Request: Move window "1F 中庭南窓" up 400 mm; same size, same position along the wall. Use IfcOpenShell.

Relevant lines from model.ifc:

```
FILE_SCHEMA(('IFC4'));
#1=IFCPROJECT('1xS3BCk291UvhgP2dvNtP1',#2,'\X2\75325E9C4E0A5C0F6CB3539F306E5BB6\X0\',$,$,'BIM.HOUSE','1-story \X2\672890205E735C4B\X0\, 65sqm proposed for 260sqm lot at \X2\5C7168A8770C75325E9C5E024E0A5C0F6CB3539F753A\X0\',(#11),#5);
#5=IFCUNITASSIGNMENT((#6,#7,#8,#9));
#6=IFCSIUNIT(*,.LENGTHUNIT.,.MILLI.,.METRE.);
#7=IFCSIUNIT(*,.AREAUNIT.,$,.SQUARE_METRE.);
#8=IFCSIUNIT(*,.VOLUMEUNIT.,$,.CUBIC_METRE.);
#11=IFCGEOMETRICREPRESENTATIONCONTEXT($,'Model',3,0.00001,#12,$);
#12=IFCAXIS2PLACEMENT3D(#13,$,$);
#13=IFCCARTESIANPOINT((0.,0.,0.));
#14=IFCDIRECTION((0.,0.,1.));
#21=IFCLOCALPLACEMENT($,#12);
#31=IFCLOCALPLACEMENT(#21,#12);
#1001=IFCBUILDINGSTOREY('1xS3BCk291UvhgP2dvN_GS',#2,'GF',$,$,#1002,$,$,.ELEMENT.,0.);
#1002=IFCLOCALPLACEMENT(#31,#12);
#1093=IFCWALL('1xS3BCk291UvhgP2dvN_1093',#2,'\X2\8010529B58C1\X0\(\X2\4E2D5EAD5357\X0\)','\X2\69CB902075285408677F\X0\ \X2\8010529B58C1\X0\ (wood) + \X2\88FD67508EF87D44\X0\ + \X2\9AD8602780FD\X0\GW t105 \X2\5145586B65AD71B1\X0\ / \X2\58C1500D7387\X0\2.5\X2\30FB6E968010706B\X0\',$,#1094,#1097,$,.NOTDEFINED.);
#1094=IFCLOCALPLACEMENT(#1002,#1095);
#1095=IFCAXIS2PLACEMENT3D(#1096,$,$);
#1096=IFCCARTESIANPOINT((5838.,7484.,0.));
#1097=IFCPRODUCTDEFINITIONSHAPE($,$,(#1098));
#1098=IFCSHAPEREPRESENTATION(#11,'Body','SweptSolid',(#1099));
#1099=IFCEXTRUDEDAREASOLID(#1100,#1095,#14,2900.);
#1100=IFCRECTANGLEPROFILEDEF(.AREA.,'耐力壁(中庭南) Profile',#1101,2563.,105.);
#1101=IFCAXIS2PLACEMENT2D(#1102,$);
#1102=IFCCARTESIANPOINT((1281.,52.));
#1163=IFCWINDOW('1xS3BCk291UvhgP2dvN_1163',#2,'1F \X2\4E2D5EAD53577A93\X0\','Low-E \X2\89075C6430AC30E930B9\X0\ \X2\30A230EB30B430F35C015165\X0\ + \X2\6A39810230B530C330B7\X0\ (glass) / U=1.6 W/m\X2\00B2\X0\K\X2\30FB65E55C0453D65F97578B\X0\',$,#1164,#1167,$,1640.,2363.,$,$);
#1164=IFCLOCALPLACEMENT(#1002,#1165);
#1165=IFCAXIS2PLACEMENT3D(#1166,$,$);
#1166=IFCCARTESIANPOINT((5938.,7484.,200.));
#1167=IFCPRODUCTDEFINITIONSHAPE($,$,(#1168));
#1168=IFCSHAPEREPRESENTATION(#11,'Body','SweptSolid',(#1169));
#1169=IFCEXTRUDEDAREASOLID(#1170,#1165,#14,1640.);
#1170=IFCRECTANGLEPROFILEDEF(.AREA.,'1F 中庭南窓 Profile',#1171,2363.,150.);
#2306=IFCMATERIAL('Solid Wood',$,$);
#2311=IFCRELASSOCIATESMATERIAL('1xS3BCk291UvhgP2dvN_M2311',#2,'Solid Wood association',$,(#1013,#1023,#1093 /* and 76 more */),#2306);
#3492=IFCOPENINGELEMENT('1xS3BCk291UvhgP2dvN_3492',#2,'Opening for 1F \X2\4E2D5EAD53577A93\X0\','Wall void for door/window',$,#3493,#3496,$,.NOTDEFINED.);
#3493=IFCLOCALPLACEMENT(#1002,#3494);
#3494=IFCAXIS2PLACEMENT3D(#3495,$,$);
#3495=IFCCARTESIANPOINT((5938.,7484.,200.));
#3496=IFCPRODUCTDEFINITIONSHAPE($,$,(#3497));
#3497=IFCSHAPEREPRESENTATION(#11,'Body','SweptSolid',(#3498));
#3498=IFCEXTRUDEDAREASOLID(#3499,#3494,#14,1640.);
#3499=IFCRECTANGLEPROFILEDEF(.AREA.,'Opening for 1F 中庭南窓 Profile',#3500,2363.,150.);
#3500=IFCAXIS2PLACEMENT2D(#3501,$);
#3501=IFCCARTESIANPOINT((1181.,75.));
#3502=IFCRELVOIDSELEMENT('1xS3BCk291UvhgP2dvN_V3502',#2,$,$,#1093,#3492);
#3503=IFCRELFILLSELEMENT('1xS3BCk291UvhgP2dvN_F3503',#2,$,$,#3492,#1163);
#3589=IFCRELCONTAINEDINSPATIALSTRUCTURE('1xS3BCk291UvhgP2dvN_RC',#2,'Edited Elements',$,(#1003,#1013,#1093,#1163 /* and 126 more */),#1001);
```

```python
import numpy as np
import ifcopenshell
import ifcopenshell.api.geometry
import ifcopenshell.util.placement
import ifcopenshell.util.unit

model = ifcopenshell.open("model.ifc")
unit_scale = ifcopenshell.util.unit.calculate_unit_scale(model)

window = model.by_id(1163)
opening = window.FillsVoids[0].RelatingOpeningElement
dz = 400.0

shift = np.array([0.0, 0.0, dz])
# The window is not placed relative to its opening, so move both.
for product in (opening, window):
    matrix = ifcopenshell.util.placement.get_local_placement(product.ObjectPlacement)
    matrix[:3, 3] += shift
    ifcopenshell.api.geometry.edit_object_placement(model, product=product, matrix=matrix, is_si=False)

print(f"moved by {dz * unit_scale:+.3f} m")

model.write("model_updated.ifc")
```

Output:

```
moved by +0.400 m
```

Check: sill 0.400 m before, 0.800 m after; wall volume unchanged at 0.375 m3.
